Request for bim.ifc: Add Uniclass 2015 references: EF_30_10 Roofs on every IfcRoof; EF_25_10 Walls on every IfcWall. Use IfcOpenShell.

First a look at what the model holds.

```python
import ifcopenshell

model = ifcopenshell.open("bim.ifc")
print(model.schema)
print("classifications:", [c.Name for c in model.by_type("IfcClassification")])
for ifc_class in ("IfcDoor", "IfcRoof", "IfcStair", "IfcWall", "IfcWindow"):
    print(ifc_class, len(model.by_type(ifc_class)))
```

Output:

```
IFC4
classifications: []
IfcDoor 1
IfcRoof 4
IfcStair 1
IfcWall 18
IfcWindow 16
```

```python
import ifcopenshell
import ifcopenshell.api.classification

model = ifcopenshell.open("bim.ifc")

system = ifcopenshell.api.classification.add_classification(model, classification="Uniclass 2015")

codes = {
    "IfcRoof": ("EF_30_10", "Roofs"),
    "IfcWall": ("EF_25_10", "Walls"),
}
for ifc_class, (code, name) in codes.items():
    products = model.by_type(ifc_class)
    ifcopenshell.api.classification.add_reference(
        model, products=products, classification=system, identification=code, name=name
    )
    print(code, len(products))

model.write("bim-out.ifc")
```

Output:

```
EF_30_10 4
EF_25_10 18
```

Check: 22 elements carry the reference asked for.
